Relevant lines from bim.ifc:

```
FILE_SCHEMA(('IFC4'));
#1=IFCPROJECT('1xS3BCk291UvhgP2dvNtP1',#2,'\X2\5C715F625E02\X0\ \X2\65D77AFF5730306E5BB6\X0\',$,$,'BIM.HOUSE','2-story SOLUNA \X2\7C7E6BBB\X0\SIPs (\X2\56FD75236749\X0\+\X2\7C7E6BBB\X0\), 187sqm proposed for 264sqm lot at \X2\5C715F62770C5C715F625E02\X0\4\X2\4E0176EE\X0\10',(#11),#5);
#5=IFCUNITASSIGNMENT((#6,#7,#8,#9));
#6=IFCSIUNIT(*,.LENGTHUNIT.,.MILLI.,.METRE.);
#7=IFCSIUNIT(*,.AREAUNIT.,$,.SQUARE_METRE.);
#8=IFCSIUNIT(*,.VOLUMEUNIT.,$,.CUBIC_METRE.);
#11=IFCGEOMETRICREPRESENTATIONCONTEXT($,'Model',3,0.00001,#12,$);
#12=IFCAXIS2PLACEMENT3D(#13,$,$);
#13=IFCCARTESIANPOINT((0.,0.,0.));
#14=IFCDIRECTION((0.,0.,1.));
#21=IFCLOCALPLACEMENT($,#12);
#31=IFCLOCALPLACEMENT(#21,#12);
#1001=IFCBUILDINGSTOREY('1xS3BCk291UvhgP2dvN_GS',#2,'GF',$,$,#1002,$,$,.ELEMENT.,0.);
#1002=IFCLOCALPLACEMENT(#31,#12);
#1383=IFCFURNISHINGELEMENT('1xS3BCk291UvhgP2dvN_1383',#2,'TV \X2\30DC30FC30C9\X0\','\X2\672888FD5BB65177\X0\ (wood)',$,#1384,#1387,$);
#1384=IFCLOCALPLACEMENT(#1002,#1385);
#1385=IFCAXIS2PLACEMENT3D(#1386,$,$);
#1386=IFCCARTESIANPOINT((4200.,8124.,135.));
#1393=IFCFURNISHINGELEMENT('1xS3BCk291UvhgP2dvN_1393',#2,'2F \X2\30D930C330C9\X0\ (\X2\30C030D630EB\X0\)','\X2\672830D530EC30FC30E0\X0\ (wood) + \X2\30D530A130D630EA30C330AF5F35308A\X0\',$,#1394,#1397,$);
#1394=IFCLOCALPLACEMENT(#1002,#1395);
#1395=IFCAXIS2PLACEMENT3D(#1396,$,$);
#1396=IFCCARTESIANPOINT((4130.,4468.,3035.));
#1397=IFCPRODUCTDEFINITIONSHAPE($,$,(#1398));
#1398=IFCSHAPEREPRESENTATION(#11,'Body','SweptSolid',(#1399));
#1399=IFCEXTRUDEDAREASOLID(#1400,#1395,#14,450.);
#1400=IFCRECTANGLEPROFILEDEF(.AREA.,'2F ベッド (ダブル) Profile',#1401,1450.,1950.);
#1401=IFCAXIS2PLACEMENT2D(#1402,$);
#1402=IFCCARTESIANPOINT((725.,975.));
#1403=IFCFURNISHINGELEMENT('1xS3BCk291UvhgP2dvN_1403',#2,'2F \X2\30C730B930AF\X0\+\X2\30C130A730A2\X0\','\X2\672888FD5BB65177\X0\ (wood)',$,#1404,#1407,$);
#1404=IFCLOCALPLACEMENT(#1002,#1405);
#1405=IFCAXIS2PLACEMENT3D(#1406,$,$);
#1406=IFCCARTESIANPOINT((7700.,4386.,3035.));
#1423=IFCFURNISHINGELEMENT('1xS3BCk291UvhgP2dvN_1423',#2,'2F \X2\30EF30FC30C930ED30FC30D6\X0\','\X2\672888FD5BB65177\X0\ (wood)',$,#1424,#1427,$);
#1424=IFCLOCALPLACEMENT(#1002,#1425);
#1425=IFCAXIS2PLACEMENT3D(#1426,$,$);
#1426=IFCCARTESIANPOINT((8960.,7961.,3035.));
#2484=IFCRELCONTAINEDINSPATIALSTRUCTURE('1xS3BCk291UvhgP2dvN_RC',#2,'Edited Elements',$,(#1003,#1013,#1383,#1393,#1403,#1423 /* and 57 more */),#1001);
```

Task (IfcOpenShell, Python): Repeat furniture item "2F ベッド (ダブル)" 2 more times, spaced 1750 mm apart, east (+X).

```python
import numpy as np
import ifcopenshell
import ifcopenshell.api.geometry
import ifcopenshell.api.root
import ifcopenshell.util.element
import ifcopenshell.util.placement

model = ifcopenshell.open("bim.ifc")


def reuse_history(source, copy):
    """copy_class also copies each property set's owner history, people and application; keep the originals."""
    for rel in copy.IsDefinedBy:
        if rel.is_a("IfcRelDefinesByProperties") and (history := rel.RelatingPropertyDefinition.OwnerHistory):
            rel.RelatingPropertyDefinition.OwnerHistory = source.OwnerHistory
            ifcopenshell.util.element.remove_deep2(model, history)


source = model.by_guid("1xS3BCk291UvhgP2dvN_1393")
base = ifcopenshell.util.placement.get_local_placement(source.ObjectPlacement)
step = np.array([1.0, 0.0, 0.0]) * 1750.0

for i in range(1, 3):
    copy = ifcopenshell.api.root.copy_class(model, product=source)
    copy.Representation = ifcopenshell.util.element.copy_deep(
        model, source.Representation, exclude=["IfcGeometricRepresentationContext", "IfcRepresentationMap"]
    )
    reuse_history(source, copy)
    matrix = base.copy()
    matrix[:3, 3] += i * step
    print("added at", matrix[:3, 3].round(3) + 0.0)
    ifcopenshell.api.geometry.edit_object_placement(model, product=copy, matrix=matrix, is_si=False)

model.write("bim_rev.ifc")
```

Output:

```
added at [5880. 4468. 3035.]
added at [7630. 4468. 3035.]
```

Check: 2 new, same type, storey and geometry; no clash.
